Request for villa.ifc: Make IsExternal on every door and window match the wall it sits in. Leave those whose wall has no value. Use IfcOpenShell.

First a look at what the model holds.

```python
import ifcopenshell
import ifcopenshell.util.element

model = ifcopenshell.open("villa.ifc")
print(model.schema)
seen = {}
for e in model.by_type("IfcDoor") + model.by_type("IfcWindow"):
    if not e.FillsVoids:
        continue
    host = e.FillsVoids[0].RelatingOpeningElement.VoidsElements[0].RelatingBuildingElement
    own = ifcopenshell.util.element.get_pset(e, f"Pset_{e.is_a()[3:].removesuffix('StandardCase')}Common", "IsExternal")
    wall = ifcopenshell.util.element.get_pset(host, "Pset_WallCommon", "IsExternal")
    seen[e.is_a(), own, wall] = seen.get((e.is_a(), own, wall), 0) + 1
for (cls, own, wall), count in sorted(seen.items(), key=str):
    print(count, cls, "IsExternal:", own, "| host wall:", wall)
```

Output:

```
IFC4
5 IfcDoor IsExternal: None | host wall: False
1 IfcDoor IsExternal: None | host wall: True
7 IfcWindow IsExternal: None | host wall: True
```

```python
import ifcopenshell
import ifcopenshell.api.pset
import ifcopenshell.util.element

model = ifcopenshell.open("villa.ifc")

count = 0
for ifc_class, pset_name in (("IfcDoor", "Pset_DoorCommon"), ("IfcWindow", "Pset_WindowCommon")):
    for e in model.by_type(ifc_class):
        if not e.FillsVoids:
            continue
        host = e.FillsVoids[0].RelatingOpeningElement.VoidsElements[0].RelatingBuildingElement
        external = ifcopenshell.util.element.get_pset(host, "Pset_WallCommon", "IsExternal")
        if external is None or ifcopenshell.util.element.get_pset(e, pset_name, "IsExternal") == external:
            continue
        pset = ifcopenshell.api.pset.add_pset(model, product=e, name=pset_name)
        ifcopenshell.api.pset.edit_pset(model, pset=pset, properties={"IsExternal": external})
        count += 1

print(count, "updated")

model.write("villa_updated.ifc")
```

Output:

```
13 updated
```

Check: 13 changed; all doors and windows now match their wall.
